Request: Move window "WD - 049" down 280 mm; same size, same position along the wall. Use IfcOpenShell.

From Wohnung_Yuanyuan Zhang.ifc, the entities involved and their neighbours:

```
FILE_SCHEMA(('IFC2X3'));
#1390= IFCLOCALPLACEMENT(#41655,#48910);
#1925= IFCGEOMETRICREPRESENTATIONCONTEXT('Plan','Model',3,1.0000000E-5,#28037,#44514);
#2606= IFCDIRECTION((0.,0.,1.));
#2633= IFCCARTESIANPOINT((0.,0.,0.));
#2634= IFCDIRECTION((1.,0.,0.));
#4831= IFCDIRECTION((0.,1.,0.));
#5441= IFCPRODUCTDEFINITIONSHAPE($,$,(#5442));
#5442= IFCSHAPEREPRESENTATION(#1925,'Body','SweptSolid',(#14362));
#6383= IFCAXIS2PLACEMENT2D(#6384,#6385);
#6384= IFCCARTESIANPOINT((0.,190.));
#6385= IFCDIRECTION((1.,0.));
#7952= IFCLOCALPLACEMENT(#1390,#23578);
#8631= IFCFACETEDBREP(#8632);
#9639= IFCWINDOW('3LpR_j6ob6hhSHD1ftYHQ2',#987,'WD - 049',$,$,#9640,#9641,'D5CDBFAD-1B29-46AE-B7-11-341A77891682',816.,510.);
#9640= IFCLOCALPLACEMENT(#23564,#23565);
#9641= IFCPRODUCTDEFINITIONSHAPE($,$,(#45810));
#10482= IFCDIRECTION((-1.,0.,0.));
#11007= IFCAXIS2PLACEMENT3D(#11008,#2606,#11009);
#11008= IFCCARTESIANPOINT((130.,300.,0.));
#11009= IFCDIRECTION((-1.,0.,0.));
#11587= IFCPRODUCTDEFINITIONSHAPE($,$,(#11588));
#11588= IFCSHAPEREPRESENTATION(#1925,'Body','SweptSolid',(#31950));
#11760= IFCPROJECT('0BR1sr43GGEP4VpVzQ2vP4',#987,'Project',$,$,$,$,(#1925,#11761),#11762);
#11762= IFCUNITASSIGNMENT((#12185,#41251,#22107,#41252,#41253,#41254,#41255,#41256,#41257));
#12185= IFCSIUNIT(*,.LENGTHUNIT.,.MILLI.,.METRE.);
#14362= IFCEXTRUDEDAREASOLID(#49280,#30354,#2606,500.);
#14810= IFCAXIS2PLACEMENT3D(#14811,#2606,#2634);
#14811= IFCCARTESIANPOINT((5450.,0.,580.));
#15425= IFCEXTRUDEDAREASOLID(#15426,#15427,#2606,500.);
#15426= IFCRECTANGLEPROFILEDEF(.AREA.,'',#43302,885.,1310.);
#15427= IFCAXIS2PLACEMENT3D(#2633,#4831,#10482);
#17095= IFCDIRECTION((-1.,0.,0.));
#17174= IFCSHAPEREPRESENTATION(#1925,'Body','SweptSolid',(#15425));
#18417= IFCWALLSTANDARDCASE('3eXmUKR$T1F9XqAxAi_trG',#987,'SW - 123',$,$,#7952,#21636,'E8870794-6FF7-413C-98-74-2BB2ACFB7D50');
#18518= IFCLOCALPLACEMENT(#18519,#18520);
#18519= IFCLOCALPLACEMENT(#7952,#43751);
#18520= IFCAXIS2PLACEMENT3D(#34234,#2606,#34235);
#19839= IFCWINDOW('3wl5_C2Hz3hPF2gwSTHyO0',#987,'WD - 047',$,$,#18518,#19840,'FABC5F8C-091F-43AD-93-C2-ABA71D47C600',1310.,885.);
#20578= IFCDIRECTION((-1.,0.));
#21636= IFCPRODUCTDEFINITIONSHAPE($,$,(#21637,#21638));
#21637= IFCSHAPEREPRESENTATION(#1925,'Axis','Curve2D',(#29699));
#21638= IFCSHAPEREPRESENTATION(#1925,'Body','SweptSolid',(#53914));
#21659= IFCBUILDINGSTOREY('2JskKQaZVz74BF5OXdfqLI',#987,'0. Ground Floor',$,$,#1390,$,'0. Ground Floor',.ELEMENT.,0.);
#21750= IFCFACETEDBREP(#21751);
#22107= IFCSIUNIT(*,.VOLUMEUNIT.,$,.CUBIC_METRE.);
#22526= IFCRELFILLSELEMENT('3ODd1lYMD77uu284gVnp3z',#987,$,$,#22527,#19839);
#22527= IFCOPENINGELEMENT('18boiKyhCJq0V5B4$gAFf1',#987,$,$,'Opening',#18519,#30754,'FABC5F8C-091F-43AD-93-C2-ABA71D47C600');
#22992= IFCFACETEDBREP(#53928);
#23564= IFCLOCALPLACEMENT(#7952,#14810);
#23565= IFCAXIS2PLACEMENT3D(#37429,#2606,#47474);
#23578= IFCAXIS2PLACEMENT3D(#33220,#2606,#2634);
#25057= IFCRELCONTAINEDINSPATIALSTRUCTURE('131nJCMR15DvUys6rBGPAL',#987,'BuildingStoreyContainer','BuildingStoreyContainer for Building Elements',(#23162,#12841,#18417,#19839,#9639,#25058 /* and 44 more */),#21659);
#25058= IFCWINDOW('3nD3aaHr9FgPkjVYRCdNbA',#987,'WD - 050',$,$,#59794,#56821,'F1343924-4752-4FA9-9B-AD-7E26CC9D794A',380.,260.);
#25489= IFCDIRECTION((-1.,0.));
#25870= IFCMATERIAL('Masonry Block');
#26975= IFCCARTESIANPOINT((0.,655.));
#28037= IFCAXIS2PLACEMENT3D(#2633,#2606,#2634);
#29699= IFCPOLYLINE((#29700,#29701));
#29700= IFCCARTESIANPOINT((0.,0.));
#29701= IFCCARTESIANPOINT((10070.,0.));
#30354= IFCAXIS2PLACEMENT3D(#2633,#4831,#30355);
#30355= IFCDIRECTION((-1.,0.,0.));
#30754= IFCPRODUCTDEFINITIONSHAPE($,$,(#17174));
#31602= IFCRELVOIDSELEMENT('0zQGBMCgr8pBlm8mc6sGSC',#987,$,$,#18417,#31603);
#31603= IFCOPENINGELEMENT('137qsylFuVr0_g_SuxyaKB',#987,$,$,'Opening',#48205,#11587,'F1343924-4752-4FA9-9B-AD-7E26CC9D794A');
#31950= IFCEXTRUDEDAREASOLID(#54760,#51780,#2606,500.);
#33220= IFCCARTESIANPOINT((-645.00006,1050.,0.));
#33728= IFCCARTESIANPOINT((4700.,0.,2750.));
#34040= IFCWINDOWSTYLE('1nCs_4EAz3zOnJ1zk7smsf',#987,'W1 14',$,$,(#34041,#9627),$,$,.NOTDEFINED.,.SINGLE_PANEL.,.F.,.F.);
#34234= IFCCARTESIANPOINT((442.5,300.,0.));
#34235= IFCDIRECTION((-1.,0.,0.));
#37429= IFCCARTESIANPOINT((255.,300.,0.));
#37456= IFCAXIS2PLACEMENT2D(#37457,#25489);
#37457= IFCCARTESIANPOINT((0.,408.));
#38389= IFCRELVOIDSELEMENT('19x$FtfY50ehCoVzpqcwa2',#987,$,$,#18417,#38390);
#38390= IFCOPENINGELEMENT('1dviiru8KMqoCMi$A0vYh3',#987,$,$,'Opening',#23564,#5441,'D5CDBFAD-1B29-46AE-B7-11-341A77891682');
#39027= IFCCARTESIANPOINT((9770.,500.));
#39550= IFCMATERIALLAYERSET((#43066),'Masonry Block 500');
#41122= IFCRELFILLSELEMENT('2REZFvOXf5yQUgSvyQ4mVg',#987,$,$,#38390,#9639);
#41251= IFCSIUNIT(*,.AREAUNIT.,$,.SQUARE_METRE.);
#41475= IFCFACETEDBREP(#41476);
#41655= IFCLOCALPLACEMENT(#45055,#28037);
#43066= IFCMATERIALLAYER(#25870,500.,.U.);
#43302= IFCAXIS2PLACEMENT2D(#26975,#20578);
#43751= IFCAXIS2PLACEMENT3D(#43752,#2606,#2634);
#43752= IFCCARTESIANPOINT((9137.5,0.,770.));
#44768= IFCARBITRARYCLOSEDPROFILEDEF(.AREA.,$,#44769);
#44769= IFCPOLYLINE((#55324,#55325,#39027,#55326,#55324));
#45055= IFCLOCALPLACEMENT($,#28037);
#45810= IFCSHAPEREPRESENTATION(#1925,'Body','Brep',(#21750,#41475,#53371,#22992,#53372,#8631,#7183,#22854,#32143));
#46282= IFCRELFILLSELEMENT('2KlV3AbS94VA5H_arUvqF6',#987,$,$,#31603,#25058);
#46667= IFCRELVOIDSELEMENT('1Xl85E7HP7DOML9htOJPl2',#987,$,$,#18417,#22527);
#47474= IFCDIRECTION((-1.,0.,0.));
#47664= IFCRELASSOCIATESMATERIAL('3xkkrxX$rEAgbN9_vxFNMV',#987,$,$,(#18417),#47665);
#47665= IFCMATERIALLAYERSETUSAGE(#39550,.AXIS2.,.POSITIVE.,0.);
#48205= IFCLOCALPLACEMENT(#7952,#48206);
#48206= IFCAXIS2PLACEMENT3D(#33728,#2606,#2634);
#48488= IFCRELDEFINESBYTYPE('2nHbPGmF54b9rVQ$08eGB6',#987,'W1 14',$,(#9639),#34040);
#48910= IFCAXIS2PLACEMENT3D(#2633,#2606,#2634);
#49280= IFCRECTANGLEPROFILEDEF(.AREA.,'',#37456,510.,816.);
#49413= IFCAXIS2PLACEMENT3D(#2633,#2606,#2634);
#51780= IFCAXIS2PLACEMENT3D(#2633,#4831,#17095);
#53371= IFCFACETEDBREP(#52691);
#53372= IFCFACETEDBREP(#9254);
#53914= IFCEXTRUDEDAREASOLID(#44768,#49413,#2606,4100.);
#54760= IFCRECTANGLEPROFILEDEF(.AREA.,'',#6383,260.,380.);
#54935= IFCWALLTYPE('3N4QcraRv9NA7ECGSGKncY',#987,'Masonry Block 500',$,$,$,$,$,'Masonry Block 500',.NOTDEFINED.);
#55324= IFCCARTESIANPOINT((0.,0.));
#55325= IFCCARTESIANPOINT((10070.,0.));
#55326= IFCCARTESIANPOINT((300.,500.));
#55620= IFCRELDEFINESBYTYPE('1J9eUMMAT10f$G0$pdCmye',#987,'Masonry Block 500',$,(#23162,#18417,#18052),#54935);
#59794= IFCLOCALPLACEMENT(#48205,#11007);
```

```python
import numpy as np
import ifcopenshell
import ifcopenshell.api.geometry
import ifcopenshell.util.placement
import ifcopenshell.util.unit

model = ifcopenshell.open("Wohnung_Yuanyuan Zhang.ifc")
unit_scale = ifcopenshell.util.unit.calculate_unit_scale(model)

window = model.by_guid("3LpR_j6ob6hhSHD1ftYHQ2")
opening = window.FillsVoids[0].RelatingOpeningElement
dz = -280.0

shift = np.array([0.0, 0.0, dz])
# The window is placed relative to its opening, so it follows when the opening moves.
matrix = ifcopenshell.util.placement.get_local_placement(opening.ObjectPlacement)
matrix[:3, 3] += shift
ifcopenshell.api.geometry.edit_object_placement(
    model, product=opening, matrix=matrix, is_si=False, should_transform_children=True
)

print(f"moved by {dz * unit_scale:+.3f} m")

model.write("Wohnung_Yuanyuan Zhang_rev.ifc")
```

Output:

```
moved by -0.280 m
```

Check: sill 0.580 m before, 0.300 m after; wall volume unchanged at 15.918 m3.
